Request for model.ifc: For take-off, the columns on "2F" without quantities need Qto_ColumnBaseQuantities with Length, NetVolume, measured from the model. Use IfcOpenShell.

First a look at what the model holds.

```python
import ifcopenshell
import ifcopenshell.util.element
import ifcopenshell.util.unit

model = ifcopenshell.open("model.ifc")
print(model.schema)
for unit_type in ("LENGTHUNIT", "AREAUNIT", "VOLUMEUNIT"):
    print(unit_type, ifcopenshell.util.unit.calculate_unit_scale(model, unit_type))
storey = next(s for s in model.by_type("IfcBuildingStorey") if s.Name == "2F")
columns = [e for e in ifcopenshell.util.element.get_decomposition(storey) if e.is_a("IfcColumn")]
for e in sorted(columns, key=lambda e: e.id()):
    print(e.id(), e.is_a(), e.Name, list(ifcopenshell.util.element.get_psets(e, qtos_only=True)), sep=" | ")
```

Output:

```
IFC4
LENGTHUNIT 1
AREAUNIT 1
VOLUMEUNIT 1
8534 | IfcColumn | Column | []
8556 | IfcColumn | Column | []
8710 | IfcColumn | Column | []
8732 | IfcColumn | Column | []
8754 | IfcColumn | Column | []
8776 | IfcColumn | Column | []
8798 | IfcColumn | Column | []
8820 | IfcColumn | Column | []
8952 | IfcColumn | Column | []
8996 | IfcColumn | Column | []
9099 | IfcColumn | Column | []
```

```python
import ifcopenshell
import ifcopenshell.api.pset
import ifcopenshell.geom
import ifcopenshell.util.element
import ifcopenshell.util.shape
import ifcopenshell.util.unit

model = ifcopenshell.open("model.ifc")
unit_scale = ifcopenshell.util.unit.calculate_unit_scale(model)
volume_scale = ifcopenshell.util.unit.calculate_unit_scale(model, "VOLUMEUNIT")
settings = ifcopenshell.geom.settings()

storey = next(s for s in model.by_type("IfcBuildingStorey") if s.Name == "2F")
columns = [e for e in ifcopenshell.util.element.get_decomposition(storey) if e.is_a("IfcColumn")]

for e in sorted(columns, key=lambda e: e.id()):
    if ifcopenshell.util.element.get_psets(e, qtos_only=True, should_inherit=False):
        continue
    # Geometry comes back in metres, in the element's own axes.
    shape = ifcopenshell.geom.create_shape(settings, e)
    values = {
        "Length": ifcopenshell.util.shape.get_z(shape.geometry) / unit_scale,
        "NetVolume": ifcopenshell.util.shape.get_volume(shape.geometry) / volume_scale,
    }
    qto = ifcopenshell.api.pset.add_qto(model, product=e, name="Qto_ColumnBaseQuantities")
    ifcopenshell.api.pset.edit_qto(model, qto=qto, properties=values)
    print(e.id(), {k: round(v, 3) for k, v in values.items()})

model.write("model-out.ifc")
```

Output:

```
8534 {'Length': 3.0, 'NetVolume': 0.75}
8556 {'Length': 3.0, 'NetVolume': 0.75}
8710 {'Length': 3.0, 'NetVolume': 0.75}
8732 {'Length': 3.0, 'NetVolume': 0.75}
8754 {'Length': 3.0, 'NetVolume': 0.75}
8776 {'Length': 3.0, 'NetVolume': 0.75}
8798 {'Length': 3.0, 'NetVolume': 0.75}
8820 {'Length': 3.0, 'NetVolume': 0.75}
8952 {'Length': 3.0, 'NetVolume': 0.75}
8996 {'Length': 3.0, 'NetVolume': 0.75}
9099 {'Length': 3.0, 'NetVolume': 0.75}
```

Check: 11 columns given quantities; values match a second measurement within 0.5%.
